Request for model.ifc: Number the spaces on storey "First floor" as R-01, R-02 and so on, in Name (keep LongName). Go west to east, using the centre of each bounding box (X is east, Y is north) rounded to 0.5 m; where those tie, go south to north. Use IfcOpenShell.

First a look at what the model holds.

```python
import ifcopenshell
import ifcopenshell.util.element
import ifcopenshell.util.placement

model = ifcopenshell.open("model.ifc")
print(model.schema)
storey = next(s for s in model.by_type("IfcBuildingStorey") if s.Name == "First floor")
spaces = [e for e in ifcopenshell.util.element.get_decomposition(storey) if e.is_a("IfcSpace")]
for e in sorted(spaces, key=lambda e: e.id()):
    origin = ifcopenshell.util.placement.get_local_placement(e.ObjectPlacement)[:3, 3]
    print(e.id(), e.Name, e.LongName, origin.round(2) + 0.0, sep=" | ")
```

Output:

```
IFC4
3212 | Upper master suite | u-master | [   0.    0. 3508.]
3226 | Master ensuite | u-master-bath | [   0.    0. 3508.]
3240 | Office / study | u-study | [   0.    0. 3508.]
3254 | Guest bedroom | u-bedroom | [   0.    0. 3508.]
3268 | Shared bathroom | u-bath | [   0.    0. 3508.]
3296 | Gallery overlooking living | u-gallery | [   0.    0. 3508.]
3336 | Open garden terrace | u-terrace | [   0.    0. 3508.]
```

```python
import ifcopenshell
import ifcopenshell.geom
import ifcopenshell.util.element
import ifcopenshell.util.shape

model = ifcopenshell.open("model.ifc")
settings = ifcopenshell.geom.settings()
settings.set("use-world-coords", True)


def centre(element):
    shape = ifcopenshell.geom.create_shape(settings, element)
    return ifcopenshell.util.shape.get_bbox_centroid(shape.geometry)


storey = next(s for s in model.by_type("IfcBuildingStorey") if s.Name == "First floor")
spaces = [e for e in ifcopenshell.util.element.get_decomposition(storey) if e.is_a("IfcSpace")]

# Insertion points can sit at a corner or the storey origin, so sort by the geometry (in metres).
centres = {e: centre(e) for e in spaces}
spaces.sort(key=lambda e: (round(centres[e][0] / 0.5), centres[e][1]))

for i, e in enumerate(spaces, start=1):
    number = f"R-{i:02d}"
    e.Name = number
    print(e.id(), number)

model.write("model_updated.ifc")
```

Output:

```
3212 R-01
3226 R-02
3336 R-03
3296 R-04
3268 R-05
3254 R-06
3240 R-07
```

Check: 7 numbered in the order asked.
